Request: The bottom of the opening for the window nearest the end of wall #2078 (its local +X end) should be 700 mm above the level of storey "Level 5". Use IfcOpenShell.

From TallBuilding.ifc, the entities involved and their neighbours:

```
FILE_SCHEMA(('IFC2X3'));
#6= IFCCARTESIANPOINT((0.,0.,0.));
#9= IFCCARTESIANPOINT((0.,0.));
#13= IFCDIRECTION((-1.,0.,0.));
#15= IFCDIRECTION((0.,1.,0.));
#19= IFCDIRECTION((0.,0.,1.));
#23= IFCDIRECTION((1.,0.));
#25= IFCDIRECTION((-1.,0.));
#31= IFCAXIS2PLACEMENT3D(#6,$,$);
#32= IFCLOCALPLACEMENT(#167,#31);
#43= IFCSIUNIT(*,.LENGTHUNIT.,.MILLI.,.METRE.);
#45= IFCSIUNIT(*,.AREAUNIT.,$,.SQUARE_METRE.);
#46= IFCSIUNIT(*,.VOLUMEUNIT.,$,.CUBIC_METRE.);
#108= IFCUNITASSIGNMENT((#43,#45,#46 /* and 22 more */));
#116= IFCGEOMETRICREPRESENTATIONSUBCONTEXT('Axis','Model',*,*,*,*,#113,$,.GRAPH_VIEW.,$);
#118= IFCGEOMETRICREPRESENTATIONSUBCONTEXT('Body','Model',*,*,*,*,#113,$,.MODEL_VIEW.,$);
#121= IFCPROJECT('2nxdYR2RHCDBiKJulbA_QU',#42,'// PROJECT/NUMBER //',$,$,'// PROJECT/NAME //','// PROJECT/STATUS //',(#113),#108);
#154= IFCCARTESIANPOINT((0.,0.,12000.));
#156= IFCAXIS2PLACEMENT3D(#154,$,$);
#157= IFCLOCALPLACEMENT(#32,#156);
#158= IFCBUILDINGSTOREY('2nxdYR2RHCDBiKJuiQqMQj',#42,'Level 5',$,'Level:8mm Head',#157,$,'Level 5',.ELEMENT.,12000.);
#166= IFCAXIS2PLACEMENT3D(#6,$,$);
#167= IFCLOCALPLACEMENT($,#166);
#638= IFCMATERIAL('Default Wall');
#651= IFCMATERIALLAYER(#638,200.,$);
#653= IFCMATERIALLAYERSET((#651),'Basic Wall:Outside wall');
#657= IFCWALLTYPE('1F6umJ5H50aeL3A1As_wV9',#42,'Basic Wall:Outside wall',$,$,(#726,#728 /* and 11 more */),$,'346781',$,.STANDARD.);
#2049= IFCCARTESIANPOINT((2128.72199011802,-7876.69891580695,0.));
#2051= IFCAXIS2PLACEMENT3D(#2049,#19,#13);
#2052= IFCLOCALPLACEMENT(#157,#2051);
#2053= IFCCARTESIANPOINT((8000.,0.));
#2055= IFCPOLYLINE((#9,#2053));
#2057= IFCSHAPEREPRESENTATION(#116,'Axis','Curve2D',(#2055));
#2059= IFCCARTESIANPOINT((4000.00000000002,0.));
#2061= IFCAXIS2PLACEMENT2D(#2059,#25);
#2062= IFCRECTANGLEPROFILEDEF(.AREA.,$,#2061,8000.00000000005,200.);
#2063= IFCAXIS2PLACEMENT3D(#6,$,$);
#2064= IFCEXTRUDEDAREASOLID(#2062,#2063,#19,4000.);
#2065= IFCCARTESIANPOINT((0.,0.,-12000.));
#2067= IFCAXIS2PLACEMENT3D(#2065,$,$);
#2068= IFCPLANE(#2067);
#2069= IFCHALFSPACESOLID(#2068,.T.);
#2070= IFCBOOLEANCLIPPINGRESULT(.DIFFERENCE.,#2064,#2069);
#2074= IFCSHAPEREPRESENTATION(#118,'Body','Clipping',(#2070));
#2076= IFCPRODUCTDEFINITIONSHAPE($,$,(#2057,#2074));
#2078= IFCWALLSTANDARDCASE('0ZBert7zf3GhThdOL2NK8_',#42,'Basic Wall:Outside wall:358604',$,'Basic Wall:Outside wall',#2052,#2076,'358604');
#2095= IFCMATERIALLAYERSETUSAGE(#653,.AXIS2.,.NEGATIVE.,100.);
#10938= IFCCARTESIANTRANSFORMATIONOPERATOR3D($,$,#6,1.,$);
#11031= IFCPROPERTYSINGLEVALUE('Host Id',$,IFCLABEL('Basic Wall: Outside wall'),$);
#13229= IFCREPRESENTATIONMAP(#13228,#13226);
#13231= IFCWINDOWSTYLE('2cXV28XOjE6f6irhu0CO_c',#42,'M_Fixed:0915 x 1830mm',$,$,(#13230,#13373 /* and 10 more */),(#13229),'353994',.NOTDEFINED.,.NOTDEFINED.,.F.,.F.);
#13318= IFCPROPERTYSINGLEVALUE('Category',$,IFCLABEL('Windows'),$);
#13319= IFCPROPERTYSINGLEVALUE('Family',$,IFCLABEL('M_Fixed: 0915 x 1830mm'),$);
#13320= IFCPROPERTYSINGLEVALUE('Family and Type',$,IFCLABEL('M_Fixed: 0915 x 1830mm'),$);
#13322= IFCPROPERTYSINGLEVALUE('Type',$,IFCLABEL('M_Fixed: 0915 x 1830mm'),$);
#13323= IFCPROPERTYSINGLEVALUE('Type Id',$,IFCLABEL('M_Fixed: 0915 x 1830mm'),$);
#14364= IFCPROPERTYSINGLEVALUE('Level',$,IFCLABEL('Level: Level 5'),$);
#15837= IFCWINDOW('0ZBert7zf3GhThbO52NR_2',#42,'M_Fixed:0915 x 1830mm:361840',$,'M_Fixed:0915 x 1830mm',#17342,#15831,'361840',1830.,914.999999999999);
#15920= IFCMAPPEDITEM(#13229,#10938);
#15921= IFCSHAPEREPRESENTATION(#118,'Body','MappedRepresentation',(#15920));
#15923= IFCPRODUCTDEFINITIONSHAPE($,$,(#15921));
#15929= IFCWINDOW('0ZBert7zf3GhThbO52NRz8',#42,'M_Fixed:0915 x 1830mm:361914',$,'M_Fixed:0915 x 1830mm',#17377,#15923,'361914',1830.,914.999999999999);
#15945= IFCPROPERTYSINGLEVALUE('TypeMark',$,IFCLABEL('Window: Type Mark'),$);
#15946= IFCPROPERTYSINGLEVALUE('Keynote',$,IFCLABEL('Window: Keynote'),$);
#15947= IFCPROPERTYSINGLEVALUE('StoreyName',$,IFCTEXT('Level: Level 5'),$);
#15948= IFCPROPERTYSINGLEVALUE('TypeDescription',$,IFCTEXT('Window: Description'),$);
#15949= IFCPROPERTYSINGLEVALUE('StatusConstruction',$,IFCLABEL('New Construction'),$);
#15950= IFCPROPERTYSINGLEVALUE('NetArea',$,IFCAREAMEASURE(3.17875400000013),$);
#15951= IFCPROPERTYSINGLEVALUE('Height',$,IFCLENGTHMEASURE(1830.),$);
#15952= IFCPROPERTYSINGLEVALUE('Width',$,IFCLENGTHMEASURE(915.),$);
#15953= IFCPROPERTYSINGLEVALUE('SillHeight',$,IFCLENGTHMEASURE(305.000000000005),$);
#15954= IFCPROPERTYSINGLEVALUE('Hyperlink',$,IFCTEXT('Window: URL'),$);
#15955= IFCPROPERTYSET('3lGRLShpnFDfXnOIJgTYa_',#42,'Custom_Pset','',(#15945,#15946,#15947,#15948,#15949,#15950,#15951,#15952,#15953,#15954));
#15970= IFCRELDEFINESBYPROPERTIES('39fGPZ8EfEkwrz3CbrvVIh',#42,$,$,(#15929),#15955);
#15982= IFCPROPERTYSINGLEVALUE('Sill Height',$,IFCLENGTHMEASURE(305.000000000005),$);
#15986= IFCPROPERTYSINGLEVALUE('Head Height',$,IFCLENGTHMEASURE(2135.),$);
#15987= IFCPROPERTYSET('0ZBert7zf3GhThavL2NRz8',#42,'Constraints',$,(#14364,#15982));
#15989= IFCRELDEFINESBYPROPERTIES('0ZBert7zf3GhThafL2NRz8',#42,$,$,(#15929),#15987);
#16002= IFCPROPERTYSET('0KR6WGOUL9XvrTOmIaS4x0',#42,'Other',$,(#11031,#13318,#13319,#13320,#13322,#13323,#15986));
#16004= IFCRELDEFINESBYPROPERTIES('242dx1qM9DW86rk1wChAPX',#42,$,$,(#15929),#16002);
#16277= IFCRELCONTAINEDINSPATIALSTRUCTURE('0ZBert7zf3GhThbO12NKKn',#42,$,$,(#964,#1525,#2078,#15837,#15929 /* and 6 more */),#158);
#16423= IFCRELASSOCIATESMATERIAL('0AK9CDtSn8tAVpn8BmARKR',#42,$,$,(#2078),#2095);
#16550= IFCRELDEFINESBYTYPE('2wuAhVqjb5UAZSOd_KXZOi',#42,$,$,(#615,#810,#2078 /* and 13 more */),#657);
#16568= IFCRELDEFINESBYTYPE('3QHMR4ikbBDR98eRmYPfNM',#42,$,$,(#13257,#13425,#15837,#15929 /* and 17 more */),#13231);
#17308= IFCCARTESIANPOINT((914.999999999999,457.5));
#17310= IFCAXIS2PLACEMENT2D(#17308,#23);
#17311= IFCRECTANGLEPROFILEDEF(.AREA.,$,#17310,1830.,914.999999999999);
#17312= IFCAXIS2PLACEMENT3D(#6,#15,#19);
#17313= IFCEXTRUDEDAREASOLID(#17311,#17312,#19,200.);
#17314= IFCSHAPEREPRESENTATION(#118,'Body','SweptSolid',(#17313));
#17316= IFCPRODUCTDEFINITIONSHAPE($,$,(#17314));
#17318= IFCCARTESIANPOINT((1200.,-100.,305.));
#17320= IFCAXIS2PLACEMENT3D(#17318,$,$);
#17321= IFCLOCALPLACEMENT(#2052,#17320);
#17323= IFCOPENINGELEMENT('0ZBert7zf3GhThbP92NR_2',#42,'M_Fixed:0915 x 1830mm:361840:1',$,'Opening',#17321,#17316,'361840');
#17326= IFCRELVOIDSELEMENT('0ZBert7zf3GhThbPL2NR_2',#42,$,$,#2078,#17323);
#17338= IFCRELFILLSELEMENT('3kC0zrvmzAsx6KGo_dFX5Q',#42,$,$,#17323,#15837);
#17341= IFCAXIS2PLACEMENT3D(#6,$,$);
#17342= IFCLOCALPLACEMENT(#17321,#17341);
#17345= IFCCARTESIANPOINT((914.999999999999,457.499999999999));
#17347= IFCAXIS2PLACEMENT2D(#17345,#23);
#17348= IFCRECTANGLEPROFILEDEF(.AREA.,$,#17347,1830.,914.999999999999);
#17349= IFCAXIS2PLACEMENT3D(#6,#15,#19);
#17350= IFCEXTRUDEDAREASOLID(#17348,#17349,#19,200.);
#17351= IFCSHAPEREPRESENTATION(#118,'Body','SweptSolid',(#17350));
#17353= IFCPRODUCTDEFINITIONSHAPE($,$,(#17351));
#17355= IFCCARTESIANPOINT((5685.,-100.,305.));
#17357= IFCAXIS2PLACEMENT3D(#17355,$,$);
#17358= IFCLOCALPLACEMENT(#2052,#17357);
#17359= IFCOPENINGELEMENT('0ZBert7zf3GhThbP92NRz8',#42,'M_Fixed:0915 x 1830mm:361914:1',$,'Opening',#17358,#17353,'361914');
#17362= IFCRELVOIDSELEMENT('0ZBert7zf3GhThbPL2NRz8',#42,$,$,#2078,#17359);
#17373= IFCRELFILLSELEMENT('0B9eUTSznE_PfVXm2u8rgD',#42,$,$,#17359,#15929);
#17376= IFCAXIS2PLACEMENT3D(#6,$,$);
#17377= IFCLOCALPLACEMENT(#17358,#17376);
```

```python
import numpy as np
import ifcopenshell
import ifcopenshell.api.geometry
import ifcopenshell.api.pset
import ifcopenshell.geom
import ifcopenshell.util.element
import ifcopenshell.util.placement
import ifcopenshell.util.shape
import ifcopenshell.util.unit

model = ifcopenshell.open("TallBuilding.ifc")
unit_scale = ifcopenshell.util.unit.calculate_unit_scale(model)

window = model.by_guid("0ZBert7zf3GhThbO52NRz8")
opening = window.FillsVoids[0].RelatingOpeningElement
storey = ifcopenshell.util.element.get_container(window, ifc_class="IfcBuildingStorey")
level = ifcopenshell.util.placement.get_local_placement(storey.ObjectPlacement)[2, 3]

# The opening's origin need not be at the sill, so measure its lowest point.
shape = ifcopenshell.geom.create_shape(ifcopenshell.geom.settings(), opening)
bottom = ifcopenshell.util.shape.get_shape_bottom_elevation(shape, shape.geometry) / unit_scale
dz = level + 700.0 - bottom

shift = np.array([0.0, 0.0, dz])
# The window is placed relative to its opening, so it follows when the opening moves.
matrix = ifcopenshell.util.placement.get_local_placement(opening.ObjectPlacement)
matrix[:3, 3] += shift
ifcopenshell.api.geometry.edit_object_placement(
    model, product=opening, matrix=matrix, is_si=False, should_transform_children=True
)

# Keep the stored heights in step.
pset = model.by_id(ifcopenshell.util.element.get_pset(window, "Custom_Pset", should_inherit=False)["id"])
ifcopenshell.api.pset.edit_pset(model, pset=pset, properties={
    "SillHeight": model.create_entity("IfcLengthMeasure", ifcopenshell.util.element.get_pset(window, "Constraints", "Sill Height") + dz),
})
pset = model.by_id(ifcopenshell.util.element.get_pset(window, "Constraints", should_inherit=False)["id"])
ifcopenshell.api.pset.edit_pset(model, pset=pset, properties={
    "Sill Height": model.create_entity("IfcLengthMeasure", ifcopenshell.util.element.get_pset(window, "Constraints", "Sill Height") + dz),
})
pset = model.by_id(ifcopenshell.util.element.get_pset(window, "Other", should_inherit=False)["id"])
ifcopenshell.api.pset.edit_pset(model, pset=pset, properties={
    "Head Height": model.create_entity("IfcLengthMeasure", ifcopenshell.util.element.get_pset(window, "Other", "Head Height") + dz),
})

print(f"moved by {dz * unit_scale:+.3f} m")

model.write("TallBuilding-out.ifc")
```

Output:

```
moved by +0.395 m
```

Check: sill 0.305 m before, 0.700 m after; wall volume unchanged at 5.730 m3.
